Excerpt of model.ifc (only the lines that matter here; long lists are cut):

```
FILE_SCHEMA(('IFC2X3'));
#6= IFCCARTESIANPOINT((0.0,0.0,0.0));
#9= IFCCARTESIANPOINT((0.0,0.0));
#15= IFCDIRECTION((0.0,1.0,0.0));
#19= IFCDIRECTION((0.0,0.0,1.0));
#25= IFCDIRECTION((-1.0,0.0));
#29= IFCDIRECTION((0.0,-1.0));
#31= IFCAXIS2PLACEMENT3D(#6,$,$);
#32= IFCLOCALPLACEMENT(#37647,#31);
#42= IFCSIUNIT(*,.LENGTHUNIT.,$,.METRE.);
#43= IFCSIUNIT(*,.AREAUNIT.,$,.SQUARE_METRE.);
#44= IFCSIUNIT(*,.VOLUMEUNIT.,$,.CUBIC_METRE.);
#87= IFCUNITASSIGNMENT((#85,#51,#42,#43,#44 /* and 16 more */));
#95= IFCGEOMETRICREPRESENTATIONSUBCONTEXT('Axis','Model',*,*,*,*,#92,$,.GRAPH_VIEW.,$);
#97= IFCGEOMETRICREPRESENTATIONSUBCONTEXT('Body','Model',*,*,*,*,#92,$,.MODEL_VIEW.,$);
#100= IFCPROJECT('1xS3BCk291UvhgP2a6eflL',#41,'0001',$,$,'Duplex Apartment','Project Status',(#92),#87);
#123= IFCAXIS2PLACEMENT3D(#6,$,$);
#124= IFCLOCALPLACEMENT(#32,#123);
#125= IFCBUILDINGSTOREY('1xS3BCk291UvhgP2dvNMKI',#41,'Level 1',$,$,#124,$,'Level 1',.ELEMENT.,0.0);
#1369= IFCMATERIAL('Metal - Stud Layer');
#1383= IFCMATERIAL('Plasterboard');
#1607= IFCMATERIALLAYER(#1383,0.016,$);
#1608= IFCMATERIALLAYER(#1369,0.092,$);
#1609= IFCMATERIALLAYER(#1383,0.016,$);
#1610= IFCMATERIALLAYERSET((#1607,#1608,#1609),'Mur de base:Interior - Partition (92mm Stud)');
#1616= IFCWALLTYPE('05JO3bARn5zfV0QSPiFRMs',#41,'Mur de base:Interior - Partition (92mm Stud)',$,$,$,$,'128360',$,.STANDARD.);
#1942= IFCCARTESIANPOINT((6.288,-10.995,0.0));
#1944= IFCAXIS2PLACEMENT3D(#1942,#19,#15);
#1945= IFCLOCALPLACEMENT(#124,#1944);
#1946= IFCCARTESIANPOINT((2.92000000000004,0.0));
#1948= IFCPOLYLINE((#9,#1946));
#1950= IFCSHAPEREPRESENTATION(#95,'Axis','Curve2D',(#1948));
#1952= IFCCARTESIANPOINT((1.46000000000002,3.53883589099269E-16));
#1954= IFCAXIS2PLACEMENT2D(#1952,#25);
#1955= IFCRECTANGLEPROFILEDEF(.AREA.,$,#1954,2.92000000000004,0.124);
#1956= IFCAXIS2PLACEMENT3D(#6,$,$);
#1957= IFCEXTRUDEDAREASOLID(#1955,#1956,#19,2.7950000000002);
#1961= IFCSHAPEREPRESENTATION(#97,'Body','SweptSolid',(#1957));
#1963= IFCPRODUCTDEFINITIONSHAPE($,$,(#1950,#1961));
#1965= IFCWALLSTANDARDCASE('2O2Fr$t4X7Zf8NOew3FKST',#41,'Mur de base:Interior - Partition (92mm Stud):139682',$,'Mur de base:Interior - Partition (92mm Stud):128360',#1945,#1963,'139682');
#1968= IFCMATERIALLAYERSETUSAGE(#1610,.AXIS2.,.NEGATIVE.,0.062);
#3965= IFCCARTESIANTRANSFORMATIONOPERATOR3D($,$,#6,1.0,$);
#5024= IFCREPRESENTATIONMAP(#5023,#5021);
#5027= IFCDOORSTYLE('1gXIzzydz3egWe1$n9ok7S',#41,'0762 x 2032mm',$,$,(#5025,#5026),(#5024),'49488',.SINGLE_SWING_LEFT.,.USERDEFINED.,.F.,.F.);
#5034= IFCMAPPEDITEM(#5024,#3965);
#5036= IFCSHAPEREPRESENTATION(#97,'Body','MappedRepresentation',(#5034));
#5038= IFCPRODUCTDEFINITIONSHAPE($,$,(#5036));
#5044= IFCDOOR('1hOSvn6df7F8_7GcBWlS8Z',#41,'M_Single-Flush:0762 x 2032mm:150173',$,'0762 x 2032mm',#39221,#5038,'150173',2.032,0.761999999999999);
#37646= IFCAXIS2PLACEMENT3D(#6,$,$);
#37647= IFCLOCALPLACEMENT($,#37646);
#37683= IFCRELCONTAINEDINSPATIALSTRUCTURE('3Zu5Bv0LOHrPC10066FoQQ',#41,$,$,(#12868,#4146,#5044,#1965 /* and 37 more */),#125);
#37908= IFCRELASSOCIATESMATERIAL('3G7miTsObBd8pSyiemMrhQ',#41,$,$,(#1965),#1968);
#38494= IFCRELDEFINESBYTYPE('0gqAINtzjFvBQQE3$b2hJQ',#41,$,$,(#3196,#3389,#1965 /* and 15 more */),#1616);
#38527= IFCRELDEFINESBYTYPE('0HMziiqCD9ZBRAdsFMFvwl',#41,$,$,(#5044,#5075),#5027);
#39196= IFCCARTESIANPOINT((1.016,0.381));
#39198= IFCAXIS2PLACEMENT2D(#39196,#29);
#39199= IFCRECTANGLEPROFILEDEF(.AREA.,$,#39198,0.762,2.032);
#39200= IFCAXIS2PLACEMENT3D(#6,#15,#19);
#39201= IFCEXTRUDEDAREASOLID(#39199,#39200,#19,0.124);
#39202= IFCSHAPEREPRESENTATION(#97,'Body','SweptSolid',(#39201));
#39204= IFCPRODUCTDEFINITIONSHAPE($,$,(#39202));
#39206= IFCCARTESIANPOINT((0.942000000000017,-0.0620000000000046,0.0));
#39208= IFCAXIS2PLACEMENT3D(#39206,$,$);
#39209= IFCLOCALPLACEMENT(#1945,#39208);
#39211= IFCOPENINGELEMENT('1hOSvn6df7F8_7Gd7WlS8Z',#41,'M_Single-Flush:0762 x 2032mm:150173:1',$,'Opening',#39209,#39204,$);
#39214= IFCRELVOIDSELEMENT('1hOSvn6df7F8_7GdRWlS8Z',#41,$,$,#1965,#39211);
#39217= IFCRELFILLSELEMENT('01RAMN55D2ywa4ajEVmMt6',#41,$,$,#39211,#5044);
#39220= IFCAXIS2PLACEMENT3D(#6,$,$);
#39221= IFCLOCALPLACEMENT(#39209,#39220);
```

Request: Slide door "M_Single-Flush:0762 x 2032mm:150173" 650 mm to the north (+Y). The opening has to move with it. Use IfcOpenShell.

```python
import ifcopenshell
import ifcopenshell.api.geometry
import ifcopenshell.util.placement
import ifcopenshell.util.unit

model = ifcopenshell.open("model.ifc")
unit_scale = ifcopenshell.util.unit.calculate_unit_scale(model)

door = model.by_guid("1hOSvn6df7F8_7GcBWlS8Z")
opening = door.FillsVoids[0].RelatingOpeningElement
wall = opening.VoidsElements[0].RelatingBuildingElement

wall_matrix = ifcopenshell.util.placement.get_local_placement(wall.ObjectPlacement)
shift = wall_matrix[:3, 0] * 0.65 / unit_scale
before = ifcopenshell.util.placement.get_local_placement(door.ObjectPlacement)[:3, 3].copy()

# The door is placed relative to its opening, so it follows when the opening moves.
matrix = ifcopenshell.util.placement.get_local_placement(opening.ObjectPlacement)
matrix[:3, 3] += shift
ifcopenshell.api.geometry.edit_object_placement(
    model, product=opening, matrix=matrix, is_si=False, should_transform_children=True
)

after = ifcopenshell.util.placement.get_local_placement(door.ObjectPlacement)[:3, 3]
print("door moved by", (after - before).round(3) + 0.0)

model.write("model_updated.ifc")
```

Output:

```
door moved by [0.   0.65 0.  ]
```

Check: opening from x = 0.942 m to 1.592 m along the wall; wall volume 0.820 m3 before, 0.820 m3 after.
